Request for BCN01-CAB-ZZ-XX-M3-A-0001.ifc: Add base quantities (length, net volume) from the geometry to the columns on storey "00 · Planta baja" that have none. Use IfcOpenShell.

First a look at what the model holds.

```python
import ifcopenshell
import ifcopenshell.util.element
import ifcopenshell.util.unit

model = ifcopenshell.open("BCN01-CAB-ZZ-XX-M3-A-0001.ifc")
print(model.schema)
for unit_type in ("LENGTHUNIT", "AREAUNIT", "VOLUMEUNIT"):
    print(unit_type, ifcopenshell.util.unit.calculate_unit_scale(model, unit_type))
storey = next(s for s in model.by_type("IfcBuildingStorey") if s.Name == "00 · Planta baja")
columns = [e for e in ifcopenshell.util.element.get_decomposition(storey) if e.is_a("IfcColumn")]
for e in sorted(columns, key=lambda e: e.id()):
    print(e.id(), e.is_a(), e.Name, list(ifcopenshell.util.element.get_psets(e, qtos_only=True)), sep=" | ")
```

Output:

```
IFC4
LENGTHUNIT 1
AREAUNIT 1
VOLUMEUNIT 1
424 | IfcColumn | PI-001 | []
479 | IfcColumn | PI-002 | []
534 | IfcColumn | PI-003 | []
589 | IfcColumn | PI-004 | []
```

```python
import ifcopenshell
import ifcopenshell.api.pset
import ifcopenshell.geom
import ifcopenshell.util.element
import ifcopenshell.util.shape
import ifcopenshell.util.unit

model = ifcopenshell.open("BCN01-CAB-ZZ-XX-M3-A-0001.ifc")
unit_scale = ifcopenshell.util.unit.calculate_unit_scale(model)
volume_scale = ifcopenshell.util.unit.calculate_unit_scale(model, "VOLUMEUNIT")
settings = ifcopenshell.geom.settings()

storey = next(s for s in model.by_type("IfcBuildingStorey") if s.Name == "00 · Planta baja")
columns = [e for e in ifcopenshell.util.element.get_decomposition(storey) if e.is_a("IfcColumn")]

for e in sorted(columns, key=lambda e: e.id()):
    if ifcopenshell.util.element.get_psets(e, qtos_only=True, should_inherit=False):
        continue
    # Geometry comes back in metres, in the element's own axes.
    shape = ifcopenshell.geom.create_shape(settings, e)
    values = {
        "Length": ifcopenshell.util.shape.get_z(shape.geometry) / unit_scale,
        "NetVolume": ifcopenshell.util.shape.get_volume(shape.geometry) / volume_scale,
    }
    qto = ifcopenshell.api.pset.add_qto(model, product=e, name="Qto_ColumnBaseQuantities")
    ifcopenshell.api.pset.edit_qto(model, qto=qto, properties=values)
    print(e.id(), {k: round(v, 3) for k, v in values.items()})

model.write("BCN01-CAB-ZZ-XX-M3-A-0001_edited.ifc")
```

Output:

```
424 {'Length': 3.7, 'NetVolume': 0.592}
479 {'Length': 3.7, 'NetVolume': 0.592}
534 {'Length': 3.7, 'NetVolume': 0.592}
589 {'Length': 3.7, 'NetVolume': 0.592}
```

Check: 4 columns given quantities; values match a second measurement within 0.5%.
